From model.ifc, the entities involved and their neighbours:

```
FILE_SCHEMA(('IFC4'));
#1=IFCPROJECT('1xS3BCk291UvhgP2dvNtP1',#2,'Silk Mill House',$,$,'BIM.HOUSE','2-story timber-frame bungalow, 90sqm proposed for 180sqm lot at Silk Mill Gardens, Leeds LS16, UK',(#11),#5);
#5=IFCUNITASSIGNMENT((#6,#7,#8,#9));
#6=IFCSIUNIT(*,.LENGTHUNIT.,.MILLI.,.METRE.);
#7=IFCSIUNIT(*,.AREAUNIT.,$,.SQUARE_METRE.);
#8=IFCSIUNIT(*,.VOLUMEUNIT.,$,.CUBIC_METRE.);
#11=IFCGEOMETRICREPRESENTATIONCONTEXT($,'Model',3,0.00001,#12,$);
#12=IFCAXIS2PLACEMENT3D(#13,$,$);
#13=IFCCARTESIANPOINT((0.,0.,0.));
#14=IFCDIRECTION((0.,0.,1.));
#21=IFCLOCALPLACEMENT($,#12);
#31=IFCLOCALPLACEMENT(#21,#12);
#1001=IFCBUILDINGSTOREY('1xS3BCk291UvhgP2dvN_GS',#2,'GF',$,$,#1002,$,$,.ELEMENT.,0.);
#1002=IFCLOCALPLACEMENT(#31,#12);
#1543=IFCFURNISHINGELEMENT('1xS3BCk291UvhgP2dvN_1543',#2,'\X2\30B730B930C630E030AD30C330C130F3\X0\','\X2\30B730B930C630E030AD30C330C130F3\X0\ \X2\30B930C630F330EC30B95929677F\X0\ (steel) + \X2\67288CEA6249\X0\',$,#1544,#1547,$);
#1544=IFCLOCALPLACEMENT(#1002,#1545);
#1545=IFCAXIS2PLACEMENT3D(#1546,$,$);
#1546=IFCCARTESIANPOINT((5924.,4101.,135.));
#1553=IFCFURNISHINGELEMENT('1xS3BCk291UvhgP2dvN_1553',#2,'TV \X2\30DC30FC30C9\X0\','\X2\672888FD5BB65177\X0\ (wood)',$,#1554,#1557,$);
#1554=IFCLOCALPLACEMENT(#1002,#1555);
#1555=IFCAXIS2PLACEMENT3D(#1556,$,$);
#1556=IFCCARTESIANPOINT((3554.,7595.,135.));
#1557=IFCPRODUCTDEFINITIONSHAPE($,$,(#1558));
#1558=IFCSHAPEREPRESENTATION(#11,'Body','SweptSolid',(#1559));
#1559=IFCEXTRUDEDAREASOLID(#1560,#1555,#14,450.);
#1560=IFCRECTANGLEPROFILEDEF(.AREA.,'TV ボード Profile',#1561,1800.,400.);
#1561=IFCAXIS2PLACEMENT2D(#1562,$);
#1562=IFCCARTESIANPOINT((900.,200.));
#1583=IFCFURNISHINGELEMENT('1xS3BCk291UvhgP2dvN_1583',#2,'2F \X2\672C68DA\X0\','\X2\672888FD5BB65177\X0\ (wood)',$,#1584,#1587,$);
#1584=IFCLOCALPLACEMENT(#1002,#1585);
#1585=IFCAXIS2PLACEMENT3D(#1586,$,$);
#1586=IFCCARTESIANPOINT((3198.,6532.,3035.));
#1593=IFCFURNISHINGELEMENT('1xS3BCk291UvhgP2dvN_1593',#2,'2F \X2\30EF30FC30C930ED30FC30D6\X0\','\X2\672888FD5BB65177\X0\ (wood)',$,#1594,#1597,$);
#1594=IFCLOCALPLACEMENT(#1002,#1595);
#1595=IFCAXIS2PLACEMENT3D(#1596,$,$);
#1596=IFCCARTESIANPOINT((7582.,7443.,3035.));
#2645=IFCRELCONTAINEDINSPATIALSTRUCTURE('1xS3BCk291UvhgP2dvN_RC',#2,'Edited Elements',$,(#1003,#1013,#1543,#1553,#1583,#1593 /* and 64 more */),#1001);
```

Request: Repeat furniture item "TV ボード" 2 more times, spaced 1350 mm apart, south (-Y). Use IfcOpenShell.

```python
import numpy as np
import ifcopenshell
import ifcopenshell.api.geometry
import ifcopenshell.api.root
import ifcopenshell.util.element
import ifcopenshell.util.placement

model = ifcopenshell.open("model.ifc")


def reuse_history(source, copy):
    """copy_class also copies each property set's owner history, people and application; keep the originals."""
    for rel in copy.IsDefinedBy:
        if rel.is_a("IfcRelDefinesByProperties") and (history := rel.RelatingPropertyDefinition.OwnerHistory):
            rel.RelatingPropertyDefinition.OwnerHistory = source.OwnerHistory
            ifcopenshell.util.element.remove_deep2(model, history)


source = model.by_guid("1xS3BCk291UvhgP2dvN_1553")
base = ifcopenshell.util.placement.get_local_placement(source.ObjectPlacement)
step = np.array([0.0, -1.0, 0.0]) * 1350.0

for i in range(1, 3):
    copy = ifcopenshell.api.root.copy_class(model, product=source)
    copy.Representation = ifcopenshell.util.element.copy_deep(
        model, source.Representation, exclude=["IfcGeometricRepresentationContext", "IfcRepresentationMap"]
    )
    reuse_history(source, copy)
    matrix = base.copy()
    matrix[:3, 3] += i * step
    print("added at", matrix[:3, 3].round(3) + 0.0)
    ifcopenshell.api.geometry.edit_object_placement(model, product=copy, matrix=matrix, is_si=False)

model.write("model_rev.ifc")
```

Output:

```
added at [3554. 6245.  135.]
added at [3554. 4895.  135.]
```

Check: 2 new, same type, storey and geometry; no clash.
